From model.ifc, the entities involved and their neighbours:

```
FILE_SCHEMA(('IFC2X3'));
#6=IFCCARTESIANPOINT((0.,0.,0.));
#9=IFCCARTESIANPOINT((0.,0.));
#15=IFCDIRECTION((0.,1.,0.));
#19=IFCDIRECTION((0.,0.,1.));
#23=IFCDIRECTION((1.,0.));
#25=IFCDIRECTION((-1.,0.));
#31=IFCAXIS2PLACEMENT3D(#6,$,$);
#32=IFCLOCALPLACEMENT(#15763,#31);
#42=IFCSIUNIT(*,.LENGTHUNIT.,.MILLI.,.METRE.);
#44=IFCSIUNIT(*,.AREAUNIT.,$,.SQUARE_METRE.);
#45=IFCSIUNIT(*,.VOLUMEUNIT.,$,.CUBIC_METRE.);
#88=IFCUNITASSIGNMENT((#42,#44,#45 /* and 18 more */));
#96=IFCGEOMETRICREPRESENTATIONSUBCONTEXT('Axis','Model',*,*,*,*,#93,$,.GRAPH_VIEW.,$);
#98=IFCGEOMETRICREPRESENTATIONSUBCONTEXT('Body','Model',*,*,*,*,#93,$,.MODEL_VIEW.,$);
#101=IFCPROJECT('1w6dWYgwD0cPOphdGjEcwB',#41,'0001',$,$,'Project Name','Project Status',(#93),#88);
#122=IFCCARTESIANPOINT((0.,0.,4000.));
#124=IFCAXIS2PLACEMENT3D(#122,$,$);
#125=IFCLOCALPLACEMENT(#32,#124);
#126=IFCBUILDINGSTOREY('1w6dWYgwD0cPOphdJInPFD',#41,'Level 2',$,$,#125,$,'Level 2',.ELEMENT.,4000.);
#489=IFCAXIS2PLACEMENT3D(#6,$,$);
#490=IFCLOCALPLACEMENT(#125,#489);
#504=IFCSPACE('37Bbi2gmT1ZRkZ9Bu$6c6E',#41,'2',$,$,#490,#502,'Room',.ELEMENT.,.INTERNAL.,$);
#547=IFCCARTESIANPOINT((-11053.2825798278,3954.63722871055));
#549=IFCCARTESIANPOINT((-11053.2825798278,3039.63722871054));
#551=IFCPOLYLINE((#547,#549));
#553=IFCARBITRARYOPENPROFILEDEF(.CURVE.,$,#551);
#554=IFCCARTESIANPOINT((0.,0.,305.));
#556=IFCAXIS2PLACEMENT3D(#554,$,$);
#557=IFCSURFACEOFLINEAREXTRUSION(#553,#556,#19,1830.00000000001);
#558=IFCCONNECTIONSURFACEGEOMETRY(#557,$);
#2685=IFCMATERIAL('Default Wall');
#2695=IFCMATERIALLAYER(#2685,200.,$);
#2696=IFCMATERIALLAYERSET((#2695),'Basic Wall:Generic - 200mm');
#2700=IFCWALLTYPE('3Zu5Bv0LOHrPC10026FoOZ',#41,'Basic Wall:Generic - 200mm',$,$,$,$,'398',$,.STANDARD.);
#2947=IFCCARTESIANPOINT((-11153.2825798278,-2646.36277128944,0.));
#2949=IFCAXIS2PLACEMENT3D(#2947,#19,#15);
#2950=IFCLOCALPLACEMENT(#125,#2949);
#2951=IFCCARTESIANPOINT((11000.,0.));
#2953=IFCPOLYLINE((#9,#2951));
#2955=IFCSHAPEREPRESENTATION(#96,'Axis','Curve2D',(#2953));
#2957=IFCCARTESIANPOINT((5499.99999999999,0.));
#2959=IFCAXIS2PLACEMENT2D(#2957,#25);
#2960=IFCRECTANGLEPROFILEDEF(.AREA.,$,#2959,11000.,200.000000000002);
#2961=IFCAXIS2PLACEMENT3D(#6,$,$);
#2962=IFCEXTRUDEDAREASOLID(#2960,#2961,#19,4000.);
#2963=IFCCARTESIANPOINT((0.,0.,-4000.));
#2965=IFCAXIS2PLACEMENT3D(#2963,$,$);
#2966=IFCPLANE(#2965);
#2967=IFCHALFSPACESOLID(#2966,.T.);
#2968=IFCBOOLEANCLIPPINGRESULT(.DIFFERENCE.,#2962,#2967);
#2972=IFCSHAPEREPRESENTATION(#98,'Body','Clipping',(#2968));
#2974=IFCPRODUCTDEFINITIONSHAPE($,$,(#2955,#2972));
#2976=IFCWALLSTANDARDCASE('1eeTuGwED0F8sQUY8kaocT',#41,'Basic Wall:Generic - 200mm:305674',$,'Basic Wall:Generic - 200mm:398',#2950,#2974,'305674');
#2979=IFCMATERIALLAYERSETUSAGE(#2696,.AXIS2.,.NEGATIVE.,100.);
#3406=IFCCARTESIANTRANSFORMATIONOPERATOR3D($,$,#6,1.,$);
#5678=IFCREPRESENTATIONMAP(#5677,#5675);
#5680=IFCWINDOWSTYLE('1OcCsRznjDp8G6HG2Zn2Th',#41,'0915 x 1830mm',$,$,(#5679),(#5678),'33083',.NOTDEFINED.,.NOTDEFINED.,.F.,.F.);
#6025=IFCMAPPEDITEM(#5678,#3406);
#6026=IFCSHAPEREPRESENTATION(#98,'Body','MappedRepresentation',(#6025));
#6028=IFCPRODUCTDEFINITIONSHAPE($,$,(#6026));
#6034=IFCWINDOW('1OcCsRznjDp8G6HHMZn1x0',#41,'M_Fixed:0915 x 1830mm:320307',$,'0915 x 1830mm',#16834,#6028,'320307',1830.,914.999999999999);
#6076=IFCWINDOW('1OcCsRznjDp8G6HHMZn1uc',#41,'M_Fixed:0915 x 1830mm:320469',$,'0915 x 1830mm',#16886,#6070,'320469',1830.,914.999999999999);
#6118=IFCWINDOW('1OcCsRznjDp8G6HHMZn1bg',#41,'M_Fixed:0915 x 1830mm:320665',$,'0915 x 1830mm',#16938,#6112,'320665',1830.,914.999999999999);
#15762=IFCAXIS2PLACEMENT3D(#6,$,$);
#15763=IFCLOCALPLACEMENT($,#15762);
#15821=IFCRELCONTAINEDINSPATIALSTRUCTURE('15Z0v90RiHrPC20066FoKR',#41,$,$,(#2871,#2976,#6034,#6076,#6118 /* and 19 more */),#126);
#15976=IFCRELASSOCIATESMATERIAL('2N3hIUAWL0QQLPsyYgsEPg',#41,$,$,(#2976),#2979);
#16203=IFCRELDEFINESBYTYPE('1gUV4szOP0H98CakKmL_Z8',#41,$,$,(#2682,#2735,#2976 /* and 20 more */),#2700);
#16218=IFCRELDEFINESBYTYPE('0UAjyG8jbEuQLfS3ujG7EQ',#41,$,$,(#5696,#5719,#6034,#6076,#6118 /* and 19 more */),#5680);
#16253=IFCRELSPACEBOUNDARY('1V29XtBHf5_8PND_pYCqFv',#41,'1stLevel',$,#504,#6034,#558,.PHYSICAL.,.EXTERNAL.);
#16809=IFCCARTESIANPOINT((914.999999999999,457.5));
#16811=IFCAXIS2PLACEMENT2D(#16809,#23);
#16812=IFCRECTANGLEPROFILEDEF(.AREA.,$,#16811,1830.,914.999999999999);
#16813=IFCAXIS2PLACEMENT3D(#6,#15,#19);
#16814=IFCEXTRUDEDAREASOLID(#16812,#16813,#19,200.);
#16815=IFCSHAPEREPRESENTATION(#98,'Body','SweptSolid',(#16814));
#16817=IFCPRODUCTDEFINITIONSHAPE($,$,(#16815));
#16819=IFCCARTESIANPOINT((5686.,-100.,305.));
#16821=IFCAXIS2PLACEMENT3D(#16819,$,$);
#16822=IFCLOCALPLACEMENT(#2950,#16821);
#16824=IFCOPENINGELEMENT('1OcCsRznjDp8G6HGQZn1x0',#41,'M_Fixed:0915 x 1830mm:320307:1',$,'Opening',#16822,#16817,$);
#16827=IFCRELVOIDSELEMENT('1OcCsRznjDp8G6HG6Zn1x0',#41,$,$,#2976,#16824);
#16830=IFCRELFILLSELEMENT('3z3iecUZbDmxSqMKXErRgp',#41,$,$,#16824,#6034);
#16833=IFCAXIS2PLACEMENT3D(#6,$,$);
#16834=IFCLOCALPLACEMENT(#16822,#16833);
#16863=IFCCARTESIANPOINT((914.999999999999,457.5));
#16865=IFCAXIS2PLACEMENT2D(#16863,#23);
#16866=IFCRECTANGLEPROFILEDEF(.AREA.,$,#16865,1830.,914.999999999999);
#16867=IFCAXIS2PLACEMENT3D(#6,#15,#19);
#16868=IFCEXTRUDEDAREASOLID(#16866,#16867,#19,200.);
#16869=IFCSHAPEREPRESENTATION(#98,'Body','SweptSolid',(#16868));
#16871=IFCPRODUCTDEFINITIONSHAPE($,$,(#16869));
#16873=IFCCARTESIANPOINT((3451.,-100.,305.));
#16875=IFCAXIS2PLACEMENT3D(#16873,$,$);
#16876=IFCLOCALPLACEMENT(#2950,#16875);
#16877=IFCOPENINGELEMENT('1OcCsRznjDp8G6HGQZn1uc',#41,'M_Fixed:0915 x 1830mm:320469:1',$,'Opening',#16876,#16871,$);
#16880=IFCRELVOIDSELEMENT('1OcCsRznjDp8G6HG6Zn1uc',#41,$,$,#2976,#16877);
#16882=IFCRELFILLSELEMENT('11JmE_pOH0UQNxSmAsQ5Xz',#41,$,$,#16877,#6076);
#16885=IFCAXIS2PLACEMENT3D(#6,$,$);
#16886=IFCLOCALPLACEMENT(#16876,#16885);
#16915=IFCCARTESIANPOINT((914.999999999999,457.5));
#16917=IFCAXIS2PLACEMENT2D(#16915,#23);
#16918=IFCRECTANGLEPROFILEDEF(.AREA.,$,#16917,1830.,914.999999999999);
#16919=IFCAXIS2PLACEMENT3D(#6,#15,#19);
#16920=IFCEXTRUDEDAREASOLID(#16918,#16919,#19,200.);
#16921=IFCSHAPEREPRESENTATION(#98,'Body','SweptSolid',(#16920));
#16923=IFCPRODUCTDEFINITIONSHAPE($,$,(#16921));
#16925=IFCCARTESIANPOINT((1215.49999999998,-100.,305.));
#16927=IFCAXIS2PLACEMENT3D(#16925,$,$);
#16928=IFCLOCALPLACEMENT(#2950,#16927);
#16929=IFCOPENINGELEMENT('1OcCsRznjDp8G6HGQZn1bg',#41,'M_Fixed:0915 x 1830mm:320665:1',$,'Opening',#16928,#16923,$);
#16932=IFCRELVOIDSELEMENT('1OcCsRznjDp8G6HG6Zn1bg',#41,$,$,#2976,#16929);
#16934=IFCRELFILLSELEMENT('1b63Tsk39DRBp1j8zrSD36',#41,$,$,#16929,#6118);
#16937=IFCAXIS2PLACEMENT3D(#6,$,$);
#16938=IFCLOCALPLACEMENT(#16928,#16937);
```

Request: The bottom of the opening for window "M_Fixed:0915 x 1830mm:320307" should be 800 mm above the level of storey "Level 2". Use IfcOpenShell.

```python
import numpy as np
import ifcopenshell
import ifcopenshell.api.geometry
import ifcopenshell.geom
import ifcopenshell.util.element
import ifcopenshell.util.placement
import ifcopenshell.util.shape
import ifcopenshell.util.unit

model = ifcopenshell.open("model.ifc")
unit_scale = ifcopenshell.util.unit.calculate_unit_scale(model)

window = model.by_guid("1OcCsRznjDp8G6HHMZn1x0")
opening = window.FillsVoids[0].RelatingOpeningElement
storey = ifcopenshell.util.element.get_container(window, ifc_class="IfcBuildingStorey")
level = ifcopenshell.util.placement.get_local_placement(storey.ObjectPlacement)[2, 3]

# The opening's origin need not be at the sill, so measure its lowest point.
shape = ifcopenshell.geom.create_shape(ifcopenshell.geom.settings(), opening)
bottom = ifcopenshell.util.shape.get_shape_bottom_elevation(shape, shape.geometry) / unit_scale
dz = level + 0.8 / unit_scale - bottom

shift = np.array([0.0, 0.0, dz])
# The window is placed relative to its opening, so it follows when the opening moves.
matrix = ifcopenshell.util.placement.get_local_placement(opening.ObjectPlacement)
matrix[:3, 3] += shift
ifcopenshell.api.geometry.edit_object_placement(
    model, product=opening, matrix=matrix, is_si=False, should_transform_children=True
)

# Space boundary surfaces are stored in each space's coordinates; move them too.
for rel in window.ProvidesBoundaries:
    if not rel.ConnectionGeometry:
        continue
    surface = rel.ConnectionGeometry.SurfaceOnRelatingElement
    space_matrix = ifcopenshell.util.placement.get_local_placement(rel.RelatingSpace.ObjectPlacement)
    point = np.array(surface.Position.Location.Coordinates) + space_matrix[:3, :3].T @ shift
    surface.Position = model.createIfcAxis2Placement3D(
        model.createIfcCartesianPoint(point.tolist()), surface.Position.Axis, surface.Position.RefDirection
    )

print(f"moved by {dz * unit_scale:+.3f} m")

model.write("model-out.ifc")
```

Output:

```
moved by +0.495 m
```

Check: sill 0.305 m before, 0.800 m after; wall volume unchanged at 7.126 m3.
